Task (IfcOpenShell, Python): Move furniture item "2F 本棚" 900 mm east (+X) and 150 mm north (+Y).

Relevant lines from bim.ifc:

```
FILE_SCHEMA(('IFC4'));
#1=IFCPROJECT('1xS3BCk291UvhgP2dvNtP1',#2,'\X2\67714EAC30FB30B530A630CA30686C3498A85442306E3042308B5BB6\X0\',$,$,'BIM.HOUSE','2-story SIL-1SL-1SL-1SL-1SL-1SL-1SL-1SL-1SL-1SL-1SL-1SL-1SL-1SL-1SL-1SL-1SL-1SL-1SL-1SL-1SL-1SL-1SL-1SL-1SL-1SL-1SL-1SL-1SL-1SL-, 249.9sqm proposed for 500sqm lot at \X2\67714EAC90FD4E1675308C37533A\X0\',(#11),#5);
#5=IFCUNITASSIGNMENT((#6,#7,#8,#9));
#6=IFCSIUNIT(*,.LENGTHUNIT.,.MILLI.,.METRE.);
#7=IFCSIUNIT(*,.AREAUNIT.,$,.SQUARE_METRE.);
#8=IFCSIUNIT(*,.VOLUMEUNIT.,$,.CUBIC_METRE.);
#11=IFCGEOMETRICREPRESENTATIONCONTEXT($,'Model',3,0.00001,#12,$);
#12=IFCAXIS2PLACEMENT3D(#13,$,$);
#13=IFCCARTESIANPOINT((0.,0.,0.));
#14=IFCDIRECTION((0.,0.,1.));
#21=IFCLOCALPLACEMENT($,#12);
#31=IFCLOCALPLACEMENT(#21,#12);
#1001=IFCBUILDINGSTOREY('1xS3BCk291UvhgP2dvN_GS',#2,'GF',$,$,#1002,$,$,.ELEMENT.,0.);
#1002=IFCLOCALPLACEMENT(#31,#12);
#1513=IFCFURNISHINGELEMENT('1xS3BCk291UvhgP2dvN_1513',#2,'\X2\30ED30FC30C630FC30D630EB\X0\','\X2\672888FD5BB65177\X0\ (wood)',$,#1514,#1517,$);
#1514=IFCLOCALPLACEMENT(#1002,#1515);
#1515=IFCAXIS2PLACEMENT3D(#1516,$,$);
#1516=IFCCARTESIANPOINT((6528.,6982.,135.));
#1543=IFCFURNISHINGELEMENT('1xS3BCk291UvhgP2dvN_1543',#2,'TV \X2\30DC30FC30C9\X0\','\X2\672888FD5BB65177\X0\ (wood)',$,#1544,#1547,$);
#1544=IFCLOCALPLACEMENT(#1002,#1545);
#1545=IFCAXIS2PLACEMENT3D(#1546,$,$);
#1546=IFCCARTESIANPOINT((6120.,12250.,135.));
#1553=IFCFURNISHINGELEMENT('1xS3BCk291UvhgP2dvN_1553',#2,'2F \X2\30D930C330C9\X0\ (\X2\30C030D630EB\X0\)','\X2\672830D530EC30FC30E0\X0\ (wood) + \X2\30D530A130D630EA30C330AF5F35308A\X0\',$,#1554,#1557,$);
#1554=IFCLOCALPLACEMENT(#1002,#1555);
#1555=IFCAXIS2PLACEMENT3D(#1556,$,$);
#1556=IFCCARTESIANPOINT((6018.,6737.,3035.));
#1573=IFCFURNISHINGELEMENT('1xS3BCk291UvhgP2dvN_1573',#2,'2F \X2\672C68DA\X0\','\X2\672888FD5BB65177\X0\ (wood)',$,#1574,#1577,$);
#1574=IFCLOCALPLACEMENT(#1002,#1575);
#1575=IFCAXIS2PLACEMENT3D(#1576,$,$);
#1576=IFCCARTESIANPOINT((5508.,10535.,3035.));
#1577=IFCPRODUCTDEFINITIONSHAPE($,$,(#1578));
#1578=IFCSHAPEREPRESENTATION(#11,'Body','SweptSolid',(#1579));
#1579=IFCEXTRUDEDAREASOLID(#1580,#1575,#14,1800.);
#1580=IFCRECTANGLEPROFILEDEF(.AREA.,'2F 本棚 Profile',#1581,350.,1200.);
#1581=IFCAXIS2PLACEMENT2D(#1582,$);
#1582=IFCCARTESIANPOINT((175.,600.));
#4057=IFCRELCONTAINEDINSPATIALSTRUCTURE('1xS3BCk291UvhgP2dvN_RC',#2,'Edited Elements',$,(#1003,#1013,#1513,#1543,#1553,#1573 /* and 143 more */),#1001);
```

```python
import ifcopenshell
import ifcopenshell.api.geometry
import ifcopenshell.util.placement
import ifcopenshell.util.unit

model = ifcopenshell.open("bim.ifc")
unit_scale = ifcopenshell.util.unit.calculate_unit_scale(model)

item = model.by_guid("1xS3BCk291UvhgP2dvN_1573")
matrix = ifcopenshell.util.placement.get_local_placement(item.ObjectPlacement)
matrix[0, 3] += 0.9 / unit_scale
matrix[1, 3] += 0.15 / unit_scale
ifcopenshell.api.geometry.edit_object_placement(model, product=item, matrix=matrix, is_si=False)

print(ifcopenshell.util.placement.get_local_placement(item.ObjectPlacement).round(3) + 0.0)

model.write("bim-out.ifc")
```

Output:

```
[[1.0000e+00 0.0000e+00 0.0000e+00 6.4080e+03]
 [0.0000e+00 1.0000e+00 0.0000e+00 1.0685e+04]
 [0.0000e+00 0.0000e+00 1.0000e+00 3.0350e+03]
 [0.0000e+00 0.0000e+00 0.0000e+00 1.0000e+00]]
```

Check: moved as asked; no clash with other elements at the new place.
